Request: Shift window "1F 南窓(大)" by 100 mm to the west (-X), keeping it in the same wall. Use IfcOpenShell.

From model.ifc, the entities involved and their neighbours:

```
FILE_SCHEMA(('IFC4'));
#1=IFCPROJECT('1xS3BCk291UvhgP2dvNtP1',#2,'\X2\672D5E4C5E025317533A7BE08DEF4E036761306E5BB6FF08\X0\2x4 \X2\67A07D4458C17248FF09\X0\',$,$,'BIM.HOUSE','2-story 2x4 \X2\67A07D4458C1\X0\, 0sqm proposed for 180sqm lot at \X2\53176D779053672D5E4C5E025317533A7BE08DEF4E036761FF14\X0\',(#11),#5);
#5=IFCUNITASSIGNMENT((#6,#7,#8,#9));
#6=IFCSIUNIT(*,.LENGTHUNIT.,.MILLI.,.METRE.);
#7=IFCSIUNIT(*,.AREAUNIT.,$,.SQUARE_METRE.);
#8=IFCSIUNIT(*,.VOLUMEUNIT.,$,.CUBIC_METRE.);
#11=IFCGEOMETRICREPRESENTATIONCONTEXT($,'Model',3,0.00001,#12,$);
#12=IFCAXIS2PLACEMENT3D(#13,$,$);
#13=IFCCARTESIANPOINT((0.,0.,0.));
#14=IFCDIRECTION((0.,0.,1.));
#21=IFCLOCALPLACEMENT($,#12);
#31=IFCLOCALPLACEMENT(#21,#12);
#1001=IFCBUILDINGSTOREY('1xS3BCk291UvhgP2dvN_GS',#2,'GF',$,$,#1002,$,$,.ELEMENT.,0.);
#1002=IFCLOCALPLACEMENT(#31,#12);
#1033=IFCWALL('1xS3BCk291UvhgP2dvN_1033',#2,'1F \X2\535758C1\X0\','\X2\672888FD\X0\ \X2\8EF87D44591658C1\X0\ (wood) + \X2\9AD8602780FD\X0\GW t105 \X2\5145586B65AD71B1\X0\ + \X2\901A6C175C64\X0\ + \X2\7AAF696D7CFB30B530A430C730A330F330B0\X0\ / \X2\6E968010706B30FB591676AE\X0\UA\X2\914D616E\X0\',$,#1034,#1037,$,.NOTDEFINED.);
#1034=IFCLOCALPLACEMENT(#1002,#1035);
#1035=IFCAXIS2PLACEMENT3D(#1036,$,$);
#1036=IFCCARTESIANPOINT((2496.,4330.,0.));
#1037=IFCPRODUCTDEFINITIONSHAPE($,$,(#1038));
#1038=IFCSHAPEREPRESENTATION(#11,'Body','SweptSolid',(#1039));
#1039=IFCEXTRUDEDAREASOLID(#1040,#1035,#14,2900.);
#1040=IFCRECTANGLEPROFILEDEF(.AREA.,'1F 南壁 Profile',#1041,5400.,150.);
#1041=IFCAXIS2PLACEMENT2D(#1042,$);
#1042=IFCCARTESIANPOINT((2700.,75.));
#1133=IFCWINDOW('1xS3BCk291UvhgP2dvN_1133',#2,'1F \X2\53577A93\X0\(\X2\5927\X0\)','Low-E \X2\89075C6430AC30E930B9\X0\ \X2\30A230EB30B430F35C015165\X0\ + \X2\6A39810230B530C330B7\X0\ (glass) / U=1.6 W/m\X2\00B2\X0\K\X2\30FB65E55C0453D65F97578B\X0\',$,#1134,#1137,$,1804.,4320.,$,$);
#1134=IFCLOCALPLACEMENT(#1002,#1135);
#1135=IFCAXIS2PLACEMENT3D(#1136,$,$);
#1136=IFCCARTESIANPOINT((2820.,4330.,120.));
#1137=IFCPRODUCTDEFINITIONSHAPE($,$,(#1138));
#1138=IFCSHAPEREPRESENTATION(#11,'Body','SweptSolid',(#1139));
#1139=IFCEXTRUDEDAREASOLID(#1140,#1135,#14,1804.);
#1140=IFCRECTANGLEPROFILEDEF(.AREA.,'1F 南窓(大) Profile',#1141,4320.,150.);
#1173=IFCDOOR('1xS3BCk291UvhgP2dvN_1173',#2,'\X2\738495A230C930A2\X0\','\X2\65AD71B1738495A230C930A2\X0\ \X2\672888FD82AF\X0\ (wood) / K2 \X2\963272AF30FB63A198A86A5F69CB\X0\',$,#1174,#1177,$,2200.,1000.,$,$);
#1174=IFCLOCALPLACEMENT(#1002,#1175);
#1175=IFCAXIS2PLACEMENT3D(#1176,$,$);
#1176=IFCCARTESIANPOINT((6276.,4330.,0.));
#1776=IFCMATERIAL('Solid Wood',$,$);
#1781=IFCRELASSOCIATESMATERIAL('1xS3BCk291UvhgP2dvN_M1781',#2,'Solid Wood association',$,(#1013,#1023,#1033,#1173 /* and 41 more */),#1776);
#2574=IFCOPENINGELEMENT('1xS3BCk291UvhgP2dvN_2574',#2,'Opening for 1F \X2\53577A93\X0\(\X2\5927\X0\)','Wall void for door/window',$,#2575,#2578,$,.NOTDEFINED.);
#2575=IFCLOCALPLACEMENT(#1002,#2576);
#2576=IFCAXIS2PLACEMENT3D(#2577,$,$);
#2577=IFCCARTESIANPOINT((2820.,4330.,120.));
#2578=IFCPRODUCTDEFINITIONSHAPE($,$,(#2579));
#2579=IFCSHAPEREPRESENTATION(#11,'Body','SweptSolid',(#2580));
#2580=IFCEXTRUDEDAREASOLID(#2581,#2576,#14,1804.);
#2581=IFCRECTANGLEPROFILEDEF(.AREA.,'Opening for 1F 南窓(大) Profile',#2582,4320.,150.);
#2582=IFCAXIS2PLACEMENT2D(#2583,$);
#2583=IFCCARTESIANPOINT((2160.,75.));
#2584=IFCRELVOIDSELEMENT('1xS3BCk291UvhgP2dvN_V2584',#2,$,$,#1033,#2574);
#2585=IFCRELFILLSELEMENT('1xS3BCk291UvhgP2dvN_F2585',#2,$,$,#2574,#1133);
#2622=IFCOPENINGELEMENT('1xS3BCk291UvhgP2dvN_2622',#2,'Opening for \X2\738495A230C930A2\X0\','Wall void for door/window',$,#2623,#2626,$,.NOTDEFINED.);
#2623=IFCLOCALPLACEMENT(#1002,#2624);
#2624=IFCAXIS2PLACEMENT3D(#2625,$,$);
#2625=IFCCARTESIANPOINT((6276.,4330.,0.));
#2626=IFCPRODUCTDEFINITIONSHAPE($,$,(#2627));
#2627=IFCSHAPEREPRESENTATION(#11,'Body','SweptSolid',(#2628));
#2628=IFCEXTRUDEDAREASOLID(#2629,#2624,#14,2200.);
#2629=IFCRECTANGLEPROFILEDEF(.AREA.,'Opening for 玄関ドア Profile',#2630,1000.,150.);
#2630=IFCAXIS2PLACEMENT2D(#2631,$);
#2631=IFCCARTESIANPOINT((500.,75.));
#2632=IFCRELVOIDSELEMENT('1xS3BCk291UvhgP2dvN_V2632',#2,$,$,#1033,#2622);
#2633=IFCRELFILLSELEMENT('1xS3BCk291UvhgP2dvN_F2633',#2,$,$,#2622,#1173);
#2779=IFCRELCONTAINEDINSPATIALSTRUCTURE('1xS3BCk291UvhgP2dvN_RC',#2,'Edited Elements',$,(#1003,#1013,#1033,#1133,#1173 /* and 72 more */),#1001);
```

```python
import ifcopenshell
import ifcopenshell.api.geometry
import ifcopenshell.util.placement
import ifcopenshell.util.unit

model = ifcopenshell.open("model.ifc")
unit_scale = ifcopenshell.util.unit.calculate_unit_scale(model)

window = model.by_guid("1xS3BCk291UvhgP2dvN_1133")
opening = window.FillsVoids[0].RelatingOpeningElement
wall = opening.VoidsElements[0].RelatingBuildingElement

wall_matrix = ifcopenshell.util.placement.get_local_placement(wall.ObjectPlacement)
shift = wall_matrix[:3, 0] * -0.1 / unit_scale
before = ifcopenshell.util.placement.get_local_placement(window.ObjectPlacement)[:3, 3].copy()

# The window is not placed relative to its opening, so move both.
for product in (opening, window):
    matrix = ifcopenshell.util.placement.get_local_placement(product.ObjectPlacement)
    matrix[:3, 3] += shift
    ifcopenshell.api.geometry.edit_object_placement(model, product=product, matrix=matrix, is_si=False)

after = ifcopenshell.util.placement.get_local_placement(window.ObjectPlacement)[:3, 3]
print("window moved by", (after - before).round(3) + 0.0)

model.write("model_edited.ifc")
```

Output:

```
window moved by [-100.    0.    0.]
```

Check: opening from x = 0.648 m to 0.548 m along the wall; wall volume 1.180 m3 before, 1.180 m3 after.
